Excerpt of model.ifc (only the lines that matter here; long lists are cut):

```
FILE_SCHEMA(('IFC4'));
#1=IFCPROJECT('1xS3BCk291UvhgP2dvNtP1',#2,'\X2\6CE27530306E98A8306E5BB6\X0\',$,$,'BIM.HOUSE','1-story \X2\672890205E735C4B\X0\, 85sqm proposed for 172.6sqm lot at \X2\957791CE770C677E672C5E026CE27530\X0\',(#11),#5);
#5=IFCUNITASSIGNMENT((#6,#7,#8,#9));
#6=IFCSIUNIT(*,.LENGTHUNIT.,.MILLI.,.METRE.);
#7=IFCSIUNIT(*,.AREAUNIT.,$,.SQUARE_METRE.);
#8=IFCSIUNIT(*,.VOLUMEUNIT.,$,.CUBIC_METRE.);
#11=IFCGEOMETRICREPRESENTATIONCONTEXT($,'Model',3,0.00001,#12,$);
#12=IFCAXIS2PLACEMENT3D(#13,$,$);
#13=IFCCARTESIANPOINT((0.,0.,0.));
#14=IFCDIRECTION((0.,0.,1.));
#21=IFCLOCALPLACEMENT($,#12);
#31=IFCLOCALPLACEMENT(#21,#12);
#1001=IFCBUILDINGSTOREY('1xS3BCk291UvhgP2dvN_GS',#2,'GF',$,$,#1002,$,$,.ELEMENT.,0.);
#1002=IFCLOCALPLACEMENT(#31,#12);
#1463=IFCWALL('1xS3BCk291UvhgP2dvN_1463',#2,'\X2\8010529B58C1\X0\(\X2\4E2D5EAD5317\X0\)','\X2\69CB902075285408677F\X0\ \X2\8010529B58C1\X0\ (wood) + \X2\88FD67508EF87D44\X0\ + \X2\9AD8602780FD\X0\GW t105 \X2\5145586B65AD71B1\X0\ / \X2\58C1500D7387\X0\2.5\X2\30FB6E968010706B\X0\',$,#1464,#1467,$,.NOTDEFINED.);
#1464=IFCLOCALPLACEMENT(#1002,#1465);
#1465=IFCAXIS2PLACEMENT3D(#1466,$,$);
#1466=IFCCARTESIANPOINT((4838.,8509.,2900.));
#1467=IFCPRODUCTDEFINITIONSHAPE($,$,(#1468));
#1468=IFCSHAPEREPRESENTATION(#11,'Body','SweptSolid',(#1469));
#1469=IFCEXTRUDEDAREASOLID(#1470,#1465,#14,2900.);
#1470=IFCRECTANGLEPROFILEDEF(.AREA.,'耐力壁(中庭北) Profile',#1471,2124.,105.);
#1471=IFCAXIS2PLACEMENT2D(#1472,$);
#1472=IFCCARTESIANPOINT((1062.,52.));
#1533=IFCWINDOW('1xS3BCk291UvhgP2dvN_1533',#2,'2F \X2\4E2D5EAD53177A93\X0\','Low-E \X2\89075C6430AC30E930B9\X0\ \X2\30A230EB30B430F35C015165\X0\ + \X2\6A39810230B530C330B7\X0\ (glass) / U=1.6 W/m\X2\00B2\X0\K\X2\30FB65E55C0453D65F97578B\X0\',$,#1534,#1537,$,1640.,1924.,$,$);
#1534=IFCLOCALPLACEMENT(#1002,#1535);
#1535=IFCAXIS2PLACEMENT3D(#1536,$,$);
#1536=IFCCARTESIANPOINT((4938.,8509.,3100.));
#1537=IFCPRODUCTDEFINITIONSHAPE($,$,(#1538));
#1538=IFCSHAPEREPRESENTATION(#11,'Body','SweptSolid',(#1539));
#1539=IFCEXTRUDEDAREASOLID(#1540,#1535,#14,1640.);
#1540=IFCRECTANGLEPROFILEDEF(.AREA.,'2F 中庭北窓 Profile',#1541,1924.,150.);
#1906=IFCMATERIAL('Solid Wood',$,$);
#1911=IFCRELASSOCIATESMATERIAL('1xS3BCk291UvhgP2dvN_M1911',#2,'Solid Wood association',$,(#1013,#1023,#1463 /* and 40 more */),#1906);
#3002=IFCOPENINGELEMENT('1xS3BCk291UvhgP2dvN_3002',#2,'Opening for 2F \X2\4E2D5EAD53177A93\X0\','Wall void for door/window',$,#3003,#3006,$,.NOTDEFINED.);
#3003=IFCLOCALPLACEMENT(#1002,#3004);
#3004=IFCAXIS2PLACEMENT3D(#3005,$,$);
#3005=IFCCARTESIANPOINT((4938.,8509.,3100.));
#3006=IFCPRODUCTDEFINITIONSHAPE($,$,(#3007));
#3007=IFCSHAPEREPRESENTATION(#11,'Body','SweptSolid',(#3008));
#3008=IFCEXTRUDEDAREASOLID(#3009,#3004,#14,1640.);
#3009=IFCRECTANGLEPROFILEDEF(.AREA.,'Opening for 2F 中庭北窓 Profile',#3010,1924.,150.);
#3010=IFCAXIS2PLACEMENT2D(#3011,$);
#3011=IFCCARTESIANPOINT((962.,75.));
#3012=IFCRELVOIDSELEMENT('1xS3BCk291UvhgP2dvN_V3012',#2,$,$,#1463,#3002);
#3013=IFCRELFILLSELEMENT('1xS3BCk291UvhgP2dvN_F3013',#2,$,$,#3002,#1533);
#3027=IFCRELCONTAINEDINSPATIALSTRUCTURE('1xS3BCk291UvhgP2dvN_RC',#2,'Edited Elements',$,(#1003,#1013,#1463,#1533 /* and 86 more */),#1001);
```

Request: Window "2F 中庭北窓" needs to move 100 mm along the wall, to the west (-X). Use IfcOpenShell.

```python
import ifcopenshell
import ifcopenshell.api.geometry
import ifcopenshell.util.placement
import ifcopenshell.util.unit

model = ifcopenshell.open("model.ifc")
unit_scale = ifcopenshell.util.unit.calculate_unit_scale(model)

window = model.by_id(1533)
opening = window.FillsVoids[0].RelatingOpeningElement
wall = opening.VoidsElements[0].RelatingBuildingElement

wall_matrix = ifcopenshell.util.placement.get_local_placement(wall.ObjectPlacement)
shift = wall_matrix[:3, 0] * -0.1 / unit_scale
before = ifcopenshell.util.placement.get_local_placement(window.ObjectPlacement)[:3, 3].copy()

# The window is not placed relative to its opening, so move both.
for product in (opening, window):
    matrix = ifcopenshell.util.placement.get_local_placement(product.ObjectPlacement)
    matrix[:3, 3] += shift
    ifcopenshell.api.geometry.edit_object_placement(model, product=product, matrix=matrix, is_si=False)

after = ifcopenshell.util.placement.get_local_placement(window.ObjectPlacement)[:3, 3]
print("window moved by", (after - before).round(3) + 0.0)

model.write("model_edited.ifc")
```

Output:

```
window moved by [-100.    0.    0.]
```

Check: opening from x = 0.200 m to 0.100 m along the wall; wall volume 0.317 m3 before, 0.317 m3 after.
